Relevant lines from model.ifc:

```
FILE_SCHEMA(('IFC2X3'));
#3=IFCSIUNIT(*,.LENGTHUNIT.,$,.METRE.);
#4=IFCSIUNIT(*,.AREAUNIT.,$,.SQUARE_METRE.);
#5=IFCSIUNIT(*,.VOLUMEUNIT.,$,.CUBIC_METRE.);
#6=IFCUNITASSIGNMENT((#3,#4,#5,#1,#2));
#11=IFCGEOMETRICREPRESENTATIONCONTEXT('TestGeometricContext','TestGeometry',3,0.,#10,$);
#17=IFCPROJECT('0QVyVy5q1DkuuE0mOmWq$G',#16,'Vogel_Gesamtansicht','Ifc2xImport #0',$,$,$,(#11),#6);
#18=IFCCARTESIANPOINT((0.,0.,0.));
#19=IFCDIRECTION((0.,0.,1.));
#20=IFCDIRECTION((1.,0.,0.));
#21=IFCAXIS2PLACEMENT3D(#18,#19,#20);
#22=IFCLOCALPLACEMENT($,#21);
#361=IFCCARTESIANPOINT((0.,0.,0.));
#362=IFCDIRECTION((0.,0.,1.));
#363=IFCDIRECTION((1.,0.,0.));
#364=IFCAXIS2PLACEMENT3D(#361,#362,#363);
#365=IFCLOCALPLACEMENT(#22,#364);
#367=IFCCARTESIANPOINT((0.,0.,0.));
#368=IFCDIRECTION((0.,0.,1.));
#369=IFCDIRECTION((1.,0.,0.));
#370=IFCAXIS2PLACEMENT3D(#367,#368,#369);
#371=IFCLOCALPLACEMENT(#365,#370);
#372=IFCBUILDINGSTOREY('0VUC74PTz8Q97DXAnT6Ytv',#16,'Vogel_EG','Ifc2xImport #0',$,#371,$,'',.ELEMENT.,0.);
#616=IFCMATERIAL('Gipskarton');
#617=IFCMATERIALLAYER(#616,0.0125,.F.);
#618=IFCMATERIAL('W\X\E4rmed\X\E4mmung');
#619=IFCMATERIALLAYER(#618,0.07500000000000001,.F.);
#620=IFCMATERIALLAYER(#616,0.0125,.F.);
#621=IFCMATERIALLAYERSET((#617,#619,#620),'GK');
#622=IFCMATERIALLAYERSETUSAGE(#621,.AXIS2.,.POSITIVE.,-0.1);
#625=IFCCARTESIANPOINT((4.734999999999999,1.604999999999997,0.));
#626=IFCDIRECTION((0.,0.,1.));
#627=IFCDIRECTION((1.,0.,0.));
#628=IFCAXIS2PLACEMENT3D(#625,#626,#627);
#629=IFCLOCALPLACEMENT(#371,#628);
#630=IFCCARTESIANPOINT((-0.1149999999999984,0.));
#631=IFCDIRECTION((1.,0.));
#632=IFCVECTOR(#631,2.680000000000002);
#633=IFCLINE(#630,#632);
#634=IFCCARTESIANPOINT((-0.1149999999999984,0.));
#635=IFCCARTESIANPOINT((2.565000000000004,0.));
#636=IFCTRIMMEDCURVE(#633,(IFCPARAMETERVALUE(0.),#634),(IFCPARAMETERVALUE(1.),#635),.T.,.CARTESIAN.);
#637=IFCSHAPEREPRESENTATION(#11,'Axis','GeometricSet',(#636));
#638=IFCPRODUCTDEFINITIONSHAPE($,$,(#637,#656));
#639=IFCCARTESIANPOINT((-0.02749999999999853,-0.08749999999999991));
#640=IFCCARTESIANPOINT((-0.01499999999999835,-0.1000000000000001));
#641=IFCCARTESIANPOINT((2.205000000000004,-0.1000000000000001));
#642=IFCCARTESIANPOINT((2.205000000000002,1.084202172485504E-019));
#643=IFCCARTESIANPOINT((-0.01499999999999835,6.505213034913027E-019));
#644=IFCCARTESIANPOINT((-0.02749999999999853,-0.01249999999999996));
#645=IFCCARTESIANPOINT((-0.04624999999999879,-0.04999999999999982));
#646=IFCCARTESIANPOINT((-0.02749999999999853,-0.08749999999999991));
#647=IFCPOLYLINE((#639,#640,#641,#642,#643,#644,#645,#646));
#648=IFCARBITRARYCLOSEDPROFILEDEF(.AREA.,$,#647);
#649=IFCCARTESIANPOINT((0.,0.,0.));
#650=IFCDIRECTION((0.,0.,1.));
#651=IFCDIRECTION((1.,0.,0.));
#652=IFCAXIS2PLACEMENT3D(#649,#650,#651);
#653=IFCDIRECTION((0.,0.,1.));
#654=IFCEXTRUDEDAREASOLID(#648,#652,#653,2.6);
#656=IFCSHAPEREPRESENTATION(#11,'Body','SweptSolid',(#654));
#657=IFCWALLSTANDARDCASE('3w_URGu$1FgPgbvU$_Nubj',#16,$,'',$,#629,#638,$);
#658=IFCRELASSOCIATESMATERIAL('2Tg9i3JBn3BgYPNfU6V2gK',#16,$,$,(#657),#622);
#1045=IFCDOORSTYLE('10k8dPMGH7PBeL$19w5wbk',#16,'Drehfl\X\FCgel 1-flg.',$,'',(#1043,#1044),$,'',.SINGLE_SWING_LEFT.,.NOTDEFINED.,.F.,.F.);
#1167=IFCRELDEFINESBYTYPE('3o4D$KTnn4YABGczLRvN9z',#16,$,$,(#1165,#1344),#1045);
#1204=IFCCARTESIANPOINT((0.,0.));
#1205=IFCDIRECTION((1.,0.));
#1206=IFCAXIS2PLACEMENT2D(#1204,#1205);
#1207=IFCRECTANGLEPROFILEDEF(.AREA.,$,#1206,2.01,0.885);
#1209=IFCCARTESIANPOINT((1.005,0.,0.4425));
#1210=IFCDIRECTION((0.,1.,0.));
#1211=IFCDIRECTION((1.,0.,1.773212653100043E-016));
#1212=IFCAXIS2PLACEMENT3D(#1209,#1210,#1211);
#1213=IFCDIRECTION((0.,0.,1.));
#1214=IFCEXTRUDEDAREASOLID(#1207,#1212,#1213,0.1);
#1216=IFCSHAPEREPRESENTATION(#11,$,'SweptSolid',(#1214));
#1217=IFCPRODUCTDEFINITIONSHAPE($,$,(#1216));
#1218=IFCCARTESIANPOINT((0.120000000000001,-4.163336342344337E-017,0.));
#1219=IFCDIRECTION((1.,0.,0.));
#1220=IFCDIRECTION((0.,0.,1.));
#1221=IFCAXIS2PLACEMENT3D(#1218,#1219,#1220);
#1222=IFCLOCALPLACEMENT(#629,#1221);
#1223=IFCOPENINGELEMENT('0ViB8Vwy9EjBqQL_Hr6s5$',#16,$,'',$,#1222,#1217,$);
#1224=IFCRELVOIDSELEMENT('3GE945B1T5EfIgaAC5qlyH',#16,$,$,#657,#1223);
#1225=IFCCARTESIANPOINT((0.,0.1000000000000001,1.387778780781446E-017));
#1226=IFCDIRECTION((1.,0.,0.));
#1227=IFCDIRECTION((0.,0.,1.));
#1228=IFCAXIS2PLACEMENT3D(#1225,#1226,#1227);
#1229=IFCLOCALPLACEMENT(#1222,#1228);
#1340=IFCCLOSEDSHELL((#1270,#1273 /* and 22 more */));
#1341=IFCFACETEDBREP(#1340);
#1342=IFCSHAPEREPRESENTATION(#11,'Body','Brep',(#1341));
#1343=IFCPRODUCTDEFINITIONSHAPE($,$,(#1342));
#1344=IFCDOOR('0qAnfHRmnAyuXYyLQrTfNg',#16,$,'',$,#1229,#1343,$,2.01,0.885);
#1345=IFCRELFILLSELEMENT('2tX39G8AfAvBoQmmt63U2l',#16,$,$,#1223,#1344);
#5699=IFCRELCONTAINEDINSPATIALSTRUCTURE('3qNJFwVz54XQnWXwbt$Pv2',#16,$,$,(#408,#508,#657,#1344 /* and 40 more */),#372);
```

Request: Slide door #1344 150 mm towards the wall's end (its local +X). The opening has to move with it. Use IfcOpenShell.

```python
import ifcopenshell
import ifcopenshell.api.geometry
import ifcopenshell.util.placement
import ifcopenshell.util.unit

model = ifcopenshell.open("model.ifc")
unit_scale = ifcopenshell.util.unit.calculate_unit_scale(model)

door = model.by_guid("0qAnfHRmnAyuXYyLQrTfNg")
opening = door.FillsVoids[0].RelatingOpeningElement
wall = opening.VoidsElements[0].RelatingBuildingElement

wall_matrix = ifcopenshell.util.placement.get_local_placement(wall.ObjectPlacement)
shift = wall_matrix[:3, 0] * 0.15 / unit_scale
before = ifcopenshell.util.placement.get_local_placement(door.ObjectPlacement)[:3, 3].copy()

# The door is placed relative to its opening, so it follows when the opening moves.
matrix = ifcopenshell.util.placement.get_local_placement(opening.ObjectPlacement)
matrix[:3, 3] += shift
ifcopenshell.api.geometry.edit_object_placement(
    model, product=opening, matrix=matrix, is_si=False, should_transform_children=True
)

after = ifcopenshell.util.placement.get_local_placement(door.ObjectPlacement)[:3, 3]
print("door moved by", (after - before).round(3) + 0.0)

model.write("model-out.ifc")
```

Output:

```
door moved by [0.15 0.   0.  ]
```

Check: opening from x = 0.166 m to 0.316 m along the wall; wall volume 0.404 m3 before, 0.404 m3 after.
